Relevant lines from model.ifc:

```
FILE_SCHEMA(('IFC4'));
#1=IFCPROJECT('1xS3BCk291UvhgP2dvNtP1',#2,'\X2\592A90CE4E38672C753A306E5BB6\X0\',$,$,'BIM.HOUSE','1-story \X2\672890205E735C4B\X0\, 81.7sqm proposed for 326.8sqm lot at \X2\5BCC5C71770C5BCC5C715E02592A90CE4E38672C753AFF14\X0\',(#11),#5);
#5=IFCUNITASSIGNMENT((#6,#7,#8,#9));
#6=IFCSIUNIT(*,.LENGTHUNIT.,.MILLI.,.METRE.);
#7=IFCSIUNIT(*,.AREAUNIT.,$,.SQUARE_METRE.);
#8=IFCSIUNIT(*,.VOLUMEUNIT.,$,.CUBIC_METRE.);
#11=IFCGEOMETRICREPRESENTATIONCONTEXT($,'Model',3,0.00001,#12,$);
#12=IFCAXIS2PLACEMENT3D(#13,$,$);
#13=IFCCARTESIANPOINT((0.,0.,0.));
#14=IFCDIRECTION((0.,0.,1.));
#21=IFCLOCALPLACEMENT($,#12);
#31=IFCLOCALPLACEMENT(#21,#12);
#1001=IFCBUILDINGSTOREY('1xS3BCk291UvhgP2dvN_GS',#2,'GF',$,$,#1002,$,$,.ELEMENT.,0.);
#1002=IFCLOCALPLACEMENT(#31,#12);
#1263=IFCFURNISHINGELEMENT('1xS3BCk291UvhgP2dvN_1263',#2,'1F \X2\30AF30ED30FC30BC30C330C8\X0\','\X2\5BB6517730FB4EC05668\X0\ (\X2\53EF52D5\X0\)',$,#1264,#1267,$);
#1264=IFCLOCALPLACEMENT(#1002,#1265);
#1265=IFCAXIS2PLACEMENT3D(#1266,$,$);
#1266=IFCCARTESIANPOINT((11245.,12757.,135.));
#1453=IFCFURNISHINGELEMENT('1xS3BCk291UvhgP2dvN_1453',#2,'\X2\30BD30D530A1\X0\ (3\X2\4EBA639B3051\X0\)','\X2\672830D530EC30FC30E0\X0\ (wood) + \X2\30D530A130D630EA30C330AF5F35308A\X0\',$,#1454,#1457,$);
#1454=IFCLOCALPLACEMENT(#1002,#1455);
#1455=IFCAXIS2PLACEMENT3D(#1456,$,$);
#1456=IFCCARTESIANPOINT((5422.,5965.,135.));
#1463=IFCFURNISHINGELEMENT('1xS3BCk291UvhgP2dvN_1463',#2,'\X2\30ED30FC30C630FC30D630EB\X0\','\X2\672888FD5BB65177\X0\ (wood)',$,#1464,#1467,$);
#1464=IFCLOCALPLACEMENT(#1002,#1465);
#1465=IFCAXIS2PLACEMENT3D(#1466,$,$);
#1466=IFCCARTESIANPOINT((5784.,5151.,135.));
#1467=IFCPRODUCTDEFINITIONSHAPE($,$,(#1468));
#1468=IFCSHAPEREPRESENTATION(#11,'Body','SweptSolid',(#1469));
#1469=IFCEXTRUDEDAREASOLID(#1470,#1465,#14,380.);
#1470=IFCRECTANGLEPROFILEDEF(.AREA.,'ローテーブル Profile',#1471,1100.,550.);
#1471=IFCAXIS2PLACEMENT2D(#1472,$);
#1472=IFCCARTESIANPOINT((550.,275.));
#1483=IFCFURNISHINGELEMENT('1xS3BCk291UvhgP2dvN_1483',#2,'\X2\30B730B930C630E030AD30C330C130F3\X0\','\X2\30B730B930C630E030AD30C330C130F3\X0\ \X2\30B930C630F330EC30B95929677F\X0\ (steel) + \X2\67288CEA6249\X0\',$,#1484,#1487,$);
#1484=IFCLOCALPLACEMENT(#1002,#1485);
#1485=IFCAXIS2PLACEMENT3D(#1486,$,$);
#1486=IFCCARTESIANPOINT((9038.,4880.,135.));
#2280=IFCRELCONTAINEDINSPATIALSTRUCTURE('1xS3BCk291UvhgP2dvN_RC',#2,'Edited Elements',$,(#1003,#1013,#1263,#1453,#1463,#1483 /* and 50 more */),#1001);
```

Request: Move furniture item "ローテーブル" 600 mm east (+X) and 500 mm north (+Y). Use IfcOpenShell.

```python
import ifcopenshell
import ifcopenshell.api.geometry
import ifcopenshell.util.placement
import ifcopenshell.util.unit

model = ifcopenshell.open("model.ifc")
unit_scale = ifcopenshell.util.unit.calculate_unit_scale(model)

item = model.by_guid("1xS3BCk291UvhgP2dvN_1463")
matrix = ifcopenshell.util.placement.get_local_placement(item.ObjectPlacement)
matrix[0, 3] += 0.6 / unit_scale
matrix[1, 3] += 0.5 / unit_scale
ifcopenshell.api.geometry.edit_object_placement(model, product=item, matrix=matrix, is_si=False)

print(ifcopenshell.util.placement.get_local_placement(item.ObjectPlacement).round(3) + 0.0)

model.write("model_edited.ifc")
```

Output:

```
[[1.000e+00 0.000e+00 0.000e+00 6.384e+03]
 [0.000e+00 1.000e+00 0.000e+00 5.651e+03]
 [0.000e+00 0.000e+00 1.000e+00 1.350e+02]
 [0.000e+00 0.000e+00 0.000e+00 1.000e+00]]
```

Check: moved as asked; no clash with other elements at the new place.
